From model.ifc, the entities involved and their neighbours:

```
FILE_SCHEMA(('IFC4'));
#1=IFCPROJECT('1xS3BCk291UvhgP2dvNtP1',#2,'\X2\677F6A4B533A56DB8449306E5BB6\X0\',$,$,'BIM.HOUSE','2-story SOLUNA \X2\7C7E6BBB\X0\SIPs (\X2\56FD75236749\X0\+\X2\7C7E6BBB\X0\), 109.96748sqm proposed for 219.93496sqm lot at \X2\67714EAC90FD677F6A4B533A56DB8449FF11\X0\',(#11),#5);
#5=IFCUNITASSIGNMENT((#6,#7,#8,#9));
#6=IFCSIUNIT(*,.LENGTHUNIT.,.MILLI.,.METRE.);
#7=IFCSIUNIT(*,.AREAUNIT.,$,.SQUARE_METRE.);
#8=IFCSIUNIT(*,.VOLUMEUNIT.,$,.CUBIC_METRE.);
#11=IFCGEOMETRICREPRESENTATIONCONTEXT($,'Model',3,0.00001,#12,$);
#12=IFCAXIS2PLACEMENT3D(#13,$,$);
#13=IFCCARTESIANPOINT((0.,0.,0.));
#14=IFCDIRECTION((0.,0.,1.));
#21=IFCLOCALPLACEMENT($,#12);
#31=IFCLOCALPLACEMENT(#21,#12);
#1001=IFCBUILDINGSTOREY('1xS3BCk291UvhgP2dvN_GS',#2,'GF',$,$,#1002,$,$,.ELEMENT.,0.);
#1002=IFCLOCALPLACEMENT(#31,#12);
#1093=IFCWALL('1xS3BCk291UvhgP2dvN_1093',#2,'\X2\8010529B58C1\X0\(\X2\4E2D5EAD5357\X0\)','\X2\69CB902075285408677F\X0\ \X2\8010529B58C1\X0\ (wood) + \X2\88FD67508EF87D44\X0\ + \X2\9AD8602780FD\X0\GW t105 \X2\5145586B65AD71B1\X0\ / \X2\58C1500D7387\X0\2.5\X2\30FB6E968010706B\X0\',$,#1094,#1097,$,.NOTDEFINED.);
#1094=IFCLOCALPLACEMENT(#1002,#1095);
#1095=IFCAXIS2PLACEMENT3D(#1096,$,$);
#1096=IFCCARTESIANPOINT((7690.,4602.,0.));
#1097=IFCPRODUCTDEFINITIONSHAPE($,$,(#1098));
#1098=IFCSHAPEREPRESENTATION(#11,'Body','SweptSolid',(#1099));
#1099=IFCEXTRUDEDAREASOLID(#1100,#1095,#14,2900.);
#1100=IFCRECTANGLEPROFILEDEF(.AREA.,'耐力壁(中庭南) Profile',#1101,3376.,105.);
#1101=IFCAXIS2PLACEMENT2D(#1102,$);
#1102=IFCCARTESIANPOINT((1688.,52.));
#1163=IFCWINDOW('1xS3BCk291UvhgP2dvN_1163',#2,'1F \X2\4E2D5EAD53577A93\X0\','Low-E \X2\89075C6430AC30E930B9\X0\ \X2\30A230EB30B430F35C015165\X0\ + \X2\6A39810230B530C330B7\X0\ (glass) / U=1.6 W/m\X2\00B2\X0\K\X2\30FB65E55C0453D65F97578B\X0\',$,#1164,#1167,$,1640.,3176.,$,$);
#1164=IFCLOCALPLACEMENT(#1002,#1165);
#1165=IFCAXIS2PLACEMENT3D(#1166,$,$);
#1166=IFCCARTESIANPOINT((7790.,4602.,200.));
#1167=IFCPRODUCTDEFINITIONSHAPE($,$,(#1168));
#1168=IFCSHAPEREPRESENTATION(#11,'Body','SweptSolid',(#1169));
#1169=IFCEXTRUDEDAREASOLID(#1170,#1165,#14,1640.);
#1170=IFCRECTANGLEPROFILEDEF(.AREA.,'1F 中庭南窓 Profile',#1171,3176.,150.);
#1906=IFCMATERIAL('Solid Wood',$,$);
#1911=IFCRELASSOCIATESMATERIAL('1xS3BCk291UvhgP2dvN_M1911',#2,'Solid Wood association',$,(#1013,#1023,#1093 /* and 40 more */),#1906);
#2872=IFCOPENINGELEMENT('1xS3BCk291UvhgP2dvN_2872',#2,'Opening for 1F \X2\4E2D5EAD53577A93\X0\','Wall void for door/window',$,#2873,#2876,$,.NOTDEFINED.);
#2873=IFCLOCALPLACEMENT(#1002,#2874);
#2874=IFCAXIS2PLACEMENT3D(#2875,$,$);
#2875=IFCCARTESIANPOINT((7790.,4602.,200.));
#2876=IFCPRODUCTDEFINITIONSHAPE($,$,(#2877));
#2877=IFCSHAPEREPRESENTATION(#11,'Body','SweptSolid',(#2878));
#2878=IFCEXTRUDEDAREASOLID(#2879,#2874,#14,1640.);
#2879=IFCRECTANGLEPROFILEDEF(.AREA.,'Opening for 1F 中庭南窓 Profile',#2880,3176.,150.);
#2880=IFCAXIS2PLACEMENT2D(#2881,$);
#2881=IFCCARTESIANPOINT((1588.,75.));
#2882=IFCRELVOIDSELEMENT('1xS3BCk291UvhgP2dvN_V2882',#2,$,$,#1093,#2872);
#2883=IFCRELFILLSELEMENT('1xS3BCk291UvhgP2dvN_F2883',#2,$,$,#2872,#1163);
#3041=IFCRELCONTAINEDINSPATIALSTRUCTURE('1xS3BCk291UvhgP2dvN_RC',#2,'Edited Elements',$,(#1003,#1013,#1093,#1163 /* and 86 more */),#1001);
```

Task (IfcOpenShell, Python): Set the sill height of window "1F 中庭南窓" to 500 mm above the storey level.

```python
import numpy as np
import ifcopenshell
import ifcopenshell.api.geometry
import ifcopenshell.geom
import ifcopenshell.util.element
import ifcopenshell.util.placement
import ifcopenshell.util.shape
import ifcopenshell.util.unit

model = ifcopenshell.open("model.ifc")
unit_scale = ifcopenshell.util.unit.calculate_unit_scale(model)

window = model.by_guid("1xS3BCk291UvhgP2dvN_1163")
opening = window.FillsVoids[0].RelatingOpeningElement
storey = ifcopenshell.util.element.get_container(window, ifc_class="IfcBuildingStorey")
level = ifcopenshell.util.placement.get_local_placement(storey.ObjectPlacement)[2, 3]

# The opening's origin need not be at the sill, so measure its lowest point.
shape = ifcopenshell.geom.create_shape(ifcopenshell.geom.settings(), opening)
bottom = ifcopenshell.util.shape.get_shape_bottom_elevation(shape, shape.geometry) / unit_scale
dz = level + 500.0 - bottom

shift = np.array([0.0, 0.0, dz])
# The window is not placed relative to its opening, so move both.
for product in (opening, window):
    matrix = ifcopenshell.util.placement.get_local_placement(product.ObjectPlacement)
    matrix[:3, 3] += shift
    ifcopenshell.api.geometry.edit_object_placement(model, product=product, matrix=matrix, is_si=False)

print(f"moved by {dz * unit_scale:+.3f} m")

model.write("model_v2.ifc")
```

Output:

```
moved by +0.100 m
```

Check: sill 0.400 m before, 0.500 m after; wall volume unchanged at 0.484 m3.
